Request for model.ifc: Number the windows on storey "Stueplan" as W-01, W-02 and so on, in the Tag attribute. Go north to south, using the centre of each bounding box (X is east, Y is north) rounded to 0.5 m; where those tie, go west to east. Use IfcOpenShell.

First a look at what the model holds.

```python
import ifcopenshell
import ifcopenshell.util.element
import ifcopenshell.util.placement

model = ifcopenshell.open("model.ifc")
print(model.schema)
storey = next(s for s in model.by_type("IfcBuildingStorey") if s.Name == "Stueplan")
windows = [e for e in ifcopenshell.util.element.get_decomposition(storey) if e.is_a("IfcWindow")]
for e in sorted(windows, key=lambda e: e.id()):
    origin = ifcopenshell.util.placement.get_local_placement(e.ObjectPlacement)[:3, 3]
    print(e.id(), e.Tag, e.Name, origin.round(2) + 0.0, sep=" | ")
```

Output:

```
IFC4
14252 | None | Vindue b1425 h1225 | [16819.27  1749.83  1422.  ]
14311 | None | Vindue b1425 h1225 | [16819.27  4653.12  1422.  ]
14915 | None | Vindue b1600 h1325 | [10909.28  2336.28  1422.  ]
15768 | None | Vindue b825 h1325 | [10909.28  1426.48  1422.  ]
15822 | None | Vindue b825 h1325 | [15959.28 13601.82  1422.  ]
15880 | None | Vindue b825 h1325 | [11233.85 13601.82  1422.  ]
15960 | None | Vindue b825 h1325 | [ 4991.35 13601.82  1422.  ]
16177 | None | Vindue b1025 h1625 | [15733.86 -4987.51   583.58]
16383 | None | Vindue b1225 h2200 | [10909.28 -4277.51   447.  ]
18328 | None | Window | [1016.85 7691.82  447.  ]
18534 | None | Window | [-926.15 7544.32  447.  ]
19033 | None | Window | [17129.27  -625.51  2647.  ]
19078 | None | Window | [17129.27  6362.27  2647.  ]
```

```python
import ifcopenshell
import ifcopenshell.geom
import ifcopenshell.util.element
import ifcopenshell.util.shape

model = ifcopenshell.open("model.ifc")
settings = ifcopenshell.geom.settings()
settings.set("use-world-coords", True)


def centre(element):
    shape = ifcopenshell.geom.create_shape(settings, element)
    return ifcopenshell.util.shape.get_bbox_centroid(shape.geometry)


storey = next(s for s in model.by_type("IfcBuildingStorey") if s.Name == "Stueplan")
windows = [e for e in ifcopenshell.util.element.get_decomposition(storey) if e.is_a("IfcWindow")]

# Insertion points can sit at a corner or the storey origin, so sort by the geometry (in metres).
centres = {e: centre(e) for e in windows}
windows.sort(key=lambda e: (-round(centres[e][1] / 0.5), centres[e][0]))

for i, e in enumerate(windows, start=1):
    number = f"W-{i:02d}"
    e.Tag = number
    print(e.id(), number)

model.write("model_v2.ifc")
```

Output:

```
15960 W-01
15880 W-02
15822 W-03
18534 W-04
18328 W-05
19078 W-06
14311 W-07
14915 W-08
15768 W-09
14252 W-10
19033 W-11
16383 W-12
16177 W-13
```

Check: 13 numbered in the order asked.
